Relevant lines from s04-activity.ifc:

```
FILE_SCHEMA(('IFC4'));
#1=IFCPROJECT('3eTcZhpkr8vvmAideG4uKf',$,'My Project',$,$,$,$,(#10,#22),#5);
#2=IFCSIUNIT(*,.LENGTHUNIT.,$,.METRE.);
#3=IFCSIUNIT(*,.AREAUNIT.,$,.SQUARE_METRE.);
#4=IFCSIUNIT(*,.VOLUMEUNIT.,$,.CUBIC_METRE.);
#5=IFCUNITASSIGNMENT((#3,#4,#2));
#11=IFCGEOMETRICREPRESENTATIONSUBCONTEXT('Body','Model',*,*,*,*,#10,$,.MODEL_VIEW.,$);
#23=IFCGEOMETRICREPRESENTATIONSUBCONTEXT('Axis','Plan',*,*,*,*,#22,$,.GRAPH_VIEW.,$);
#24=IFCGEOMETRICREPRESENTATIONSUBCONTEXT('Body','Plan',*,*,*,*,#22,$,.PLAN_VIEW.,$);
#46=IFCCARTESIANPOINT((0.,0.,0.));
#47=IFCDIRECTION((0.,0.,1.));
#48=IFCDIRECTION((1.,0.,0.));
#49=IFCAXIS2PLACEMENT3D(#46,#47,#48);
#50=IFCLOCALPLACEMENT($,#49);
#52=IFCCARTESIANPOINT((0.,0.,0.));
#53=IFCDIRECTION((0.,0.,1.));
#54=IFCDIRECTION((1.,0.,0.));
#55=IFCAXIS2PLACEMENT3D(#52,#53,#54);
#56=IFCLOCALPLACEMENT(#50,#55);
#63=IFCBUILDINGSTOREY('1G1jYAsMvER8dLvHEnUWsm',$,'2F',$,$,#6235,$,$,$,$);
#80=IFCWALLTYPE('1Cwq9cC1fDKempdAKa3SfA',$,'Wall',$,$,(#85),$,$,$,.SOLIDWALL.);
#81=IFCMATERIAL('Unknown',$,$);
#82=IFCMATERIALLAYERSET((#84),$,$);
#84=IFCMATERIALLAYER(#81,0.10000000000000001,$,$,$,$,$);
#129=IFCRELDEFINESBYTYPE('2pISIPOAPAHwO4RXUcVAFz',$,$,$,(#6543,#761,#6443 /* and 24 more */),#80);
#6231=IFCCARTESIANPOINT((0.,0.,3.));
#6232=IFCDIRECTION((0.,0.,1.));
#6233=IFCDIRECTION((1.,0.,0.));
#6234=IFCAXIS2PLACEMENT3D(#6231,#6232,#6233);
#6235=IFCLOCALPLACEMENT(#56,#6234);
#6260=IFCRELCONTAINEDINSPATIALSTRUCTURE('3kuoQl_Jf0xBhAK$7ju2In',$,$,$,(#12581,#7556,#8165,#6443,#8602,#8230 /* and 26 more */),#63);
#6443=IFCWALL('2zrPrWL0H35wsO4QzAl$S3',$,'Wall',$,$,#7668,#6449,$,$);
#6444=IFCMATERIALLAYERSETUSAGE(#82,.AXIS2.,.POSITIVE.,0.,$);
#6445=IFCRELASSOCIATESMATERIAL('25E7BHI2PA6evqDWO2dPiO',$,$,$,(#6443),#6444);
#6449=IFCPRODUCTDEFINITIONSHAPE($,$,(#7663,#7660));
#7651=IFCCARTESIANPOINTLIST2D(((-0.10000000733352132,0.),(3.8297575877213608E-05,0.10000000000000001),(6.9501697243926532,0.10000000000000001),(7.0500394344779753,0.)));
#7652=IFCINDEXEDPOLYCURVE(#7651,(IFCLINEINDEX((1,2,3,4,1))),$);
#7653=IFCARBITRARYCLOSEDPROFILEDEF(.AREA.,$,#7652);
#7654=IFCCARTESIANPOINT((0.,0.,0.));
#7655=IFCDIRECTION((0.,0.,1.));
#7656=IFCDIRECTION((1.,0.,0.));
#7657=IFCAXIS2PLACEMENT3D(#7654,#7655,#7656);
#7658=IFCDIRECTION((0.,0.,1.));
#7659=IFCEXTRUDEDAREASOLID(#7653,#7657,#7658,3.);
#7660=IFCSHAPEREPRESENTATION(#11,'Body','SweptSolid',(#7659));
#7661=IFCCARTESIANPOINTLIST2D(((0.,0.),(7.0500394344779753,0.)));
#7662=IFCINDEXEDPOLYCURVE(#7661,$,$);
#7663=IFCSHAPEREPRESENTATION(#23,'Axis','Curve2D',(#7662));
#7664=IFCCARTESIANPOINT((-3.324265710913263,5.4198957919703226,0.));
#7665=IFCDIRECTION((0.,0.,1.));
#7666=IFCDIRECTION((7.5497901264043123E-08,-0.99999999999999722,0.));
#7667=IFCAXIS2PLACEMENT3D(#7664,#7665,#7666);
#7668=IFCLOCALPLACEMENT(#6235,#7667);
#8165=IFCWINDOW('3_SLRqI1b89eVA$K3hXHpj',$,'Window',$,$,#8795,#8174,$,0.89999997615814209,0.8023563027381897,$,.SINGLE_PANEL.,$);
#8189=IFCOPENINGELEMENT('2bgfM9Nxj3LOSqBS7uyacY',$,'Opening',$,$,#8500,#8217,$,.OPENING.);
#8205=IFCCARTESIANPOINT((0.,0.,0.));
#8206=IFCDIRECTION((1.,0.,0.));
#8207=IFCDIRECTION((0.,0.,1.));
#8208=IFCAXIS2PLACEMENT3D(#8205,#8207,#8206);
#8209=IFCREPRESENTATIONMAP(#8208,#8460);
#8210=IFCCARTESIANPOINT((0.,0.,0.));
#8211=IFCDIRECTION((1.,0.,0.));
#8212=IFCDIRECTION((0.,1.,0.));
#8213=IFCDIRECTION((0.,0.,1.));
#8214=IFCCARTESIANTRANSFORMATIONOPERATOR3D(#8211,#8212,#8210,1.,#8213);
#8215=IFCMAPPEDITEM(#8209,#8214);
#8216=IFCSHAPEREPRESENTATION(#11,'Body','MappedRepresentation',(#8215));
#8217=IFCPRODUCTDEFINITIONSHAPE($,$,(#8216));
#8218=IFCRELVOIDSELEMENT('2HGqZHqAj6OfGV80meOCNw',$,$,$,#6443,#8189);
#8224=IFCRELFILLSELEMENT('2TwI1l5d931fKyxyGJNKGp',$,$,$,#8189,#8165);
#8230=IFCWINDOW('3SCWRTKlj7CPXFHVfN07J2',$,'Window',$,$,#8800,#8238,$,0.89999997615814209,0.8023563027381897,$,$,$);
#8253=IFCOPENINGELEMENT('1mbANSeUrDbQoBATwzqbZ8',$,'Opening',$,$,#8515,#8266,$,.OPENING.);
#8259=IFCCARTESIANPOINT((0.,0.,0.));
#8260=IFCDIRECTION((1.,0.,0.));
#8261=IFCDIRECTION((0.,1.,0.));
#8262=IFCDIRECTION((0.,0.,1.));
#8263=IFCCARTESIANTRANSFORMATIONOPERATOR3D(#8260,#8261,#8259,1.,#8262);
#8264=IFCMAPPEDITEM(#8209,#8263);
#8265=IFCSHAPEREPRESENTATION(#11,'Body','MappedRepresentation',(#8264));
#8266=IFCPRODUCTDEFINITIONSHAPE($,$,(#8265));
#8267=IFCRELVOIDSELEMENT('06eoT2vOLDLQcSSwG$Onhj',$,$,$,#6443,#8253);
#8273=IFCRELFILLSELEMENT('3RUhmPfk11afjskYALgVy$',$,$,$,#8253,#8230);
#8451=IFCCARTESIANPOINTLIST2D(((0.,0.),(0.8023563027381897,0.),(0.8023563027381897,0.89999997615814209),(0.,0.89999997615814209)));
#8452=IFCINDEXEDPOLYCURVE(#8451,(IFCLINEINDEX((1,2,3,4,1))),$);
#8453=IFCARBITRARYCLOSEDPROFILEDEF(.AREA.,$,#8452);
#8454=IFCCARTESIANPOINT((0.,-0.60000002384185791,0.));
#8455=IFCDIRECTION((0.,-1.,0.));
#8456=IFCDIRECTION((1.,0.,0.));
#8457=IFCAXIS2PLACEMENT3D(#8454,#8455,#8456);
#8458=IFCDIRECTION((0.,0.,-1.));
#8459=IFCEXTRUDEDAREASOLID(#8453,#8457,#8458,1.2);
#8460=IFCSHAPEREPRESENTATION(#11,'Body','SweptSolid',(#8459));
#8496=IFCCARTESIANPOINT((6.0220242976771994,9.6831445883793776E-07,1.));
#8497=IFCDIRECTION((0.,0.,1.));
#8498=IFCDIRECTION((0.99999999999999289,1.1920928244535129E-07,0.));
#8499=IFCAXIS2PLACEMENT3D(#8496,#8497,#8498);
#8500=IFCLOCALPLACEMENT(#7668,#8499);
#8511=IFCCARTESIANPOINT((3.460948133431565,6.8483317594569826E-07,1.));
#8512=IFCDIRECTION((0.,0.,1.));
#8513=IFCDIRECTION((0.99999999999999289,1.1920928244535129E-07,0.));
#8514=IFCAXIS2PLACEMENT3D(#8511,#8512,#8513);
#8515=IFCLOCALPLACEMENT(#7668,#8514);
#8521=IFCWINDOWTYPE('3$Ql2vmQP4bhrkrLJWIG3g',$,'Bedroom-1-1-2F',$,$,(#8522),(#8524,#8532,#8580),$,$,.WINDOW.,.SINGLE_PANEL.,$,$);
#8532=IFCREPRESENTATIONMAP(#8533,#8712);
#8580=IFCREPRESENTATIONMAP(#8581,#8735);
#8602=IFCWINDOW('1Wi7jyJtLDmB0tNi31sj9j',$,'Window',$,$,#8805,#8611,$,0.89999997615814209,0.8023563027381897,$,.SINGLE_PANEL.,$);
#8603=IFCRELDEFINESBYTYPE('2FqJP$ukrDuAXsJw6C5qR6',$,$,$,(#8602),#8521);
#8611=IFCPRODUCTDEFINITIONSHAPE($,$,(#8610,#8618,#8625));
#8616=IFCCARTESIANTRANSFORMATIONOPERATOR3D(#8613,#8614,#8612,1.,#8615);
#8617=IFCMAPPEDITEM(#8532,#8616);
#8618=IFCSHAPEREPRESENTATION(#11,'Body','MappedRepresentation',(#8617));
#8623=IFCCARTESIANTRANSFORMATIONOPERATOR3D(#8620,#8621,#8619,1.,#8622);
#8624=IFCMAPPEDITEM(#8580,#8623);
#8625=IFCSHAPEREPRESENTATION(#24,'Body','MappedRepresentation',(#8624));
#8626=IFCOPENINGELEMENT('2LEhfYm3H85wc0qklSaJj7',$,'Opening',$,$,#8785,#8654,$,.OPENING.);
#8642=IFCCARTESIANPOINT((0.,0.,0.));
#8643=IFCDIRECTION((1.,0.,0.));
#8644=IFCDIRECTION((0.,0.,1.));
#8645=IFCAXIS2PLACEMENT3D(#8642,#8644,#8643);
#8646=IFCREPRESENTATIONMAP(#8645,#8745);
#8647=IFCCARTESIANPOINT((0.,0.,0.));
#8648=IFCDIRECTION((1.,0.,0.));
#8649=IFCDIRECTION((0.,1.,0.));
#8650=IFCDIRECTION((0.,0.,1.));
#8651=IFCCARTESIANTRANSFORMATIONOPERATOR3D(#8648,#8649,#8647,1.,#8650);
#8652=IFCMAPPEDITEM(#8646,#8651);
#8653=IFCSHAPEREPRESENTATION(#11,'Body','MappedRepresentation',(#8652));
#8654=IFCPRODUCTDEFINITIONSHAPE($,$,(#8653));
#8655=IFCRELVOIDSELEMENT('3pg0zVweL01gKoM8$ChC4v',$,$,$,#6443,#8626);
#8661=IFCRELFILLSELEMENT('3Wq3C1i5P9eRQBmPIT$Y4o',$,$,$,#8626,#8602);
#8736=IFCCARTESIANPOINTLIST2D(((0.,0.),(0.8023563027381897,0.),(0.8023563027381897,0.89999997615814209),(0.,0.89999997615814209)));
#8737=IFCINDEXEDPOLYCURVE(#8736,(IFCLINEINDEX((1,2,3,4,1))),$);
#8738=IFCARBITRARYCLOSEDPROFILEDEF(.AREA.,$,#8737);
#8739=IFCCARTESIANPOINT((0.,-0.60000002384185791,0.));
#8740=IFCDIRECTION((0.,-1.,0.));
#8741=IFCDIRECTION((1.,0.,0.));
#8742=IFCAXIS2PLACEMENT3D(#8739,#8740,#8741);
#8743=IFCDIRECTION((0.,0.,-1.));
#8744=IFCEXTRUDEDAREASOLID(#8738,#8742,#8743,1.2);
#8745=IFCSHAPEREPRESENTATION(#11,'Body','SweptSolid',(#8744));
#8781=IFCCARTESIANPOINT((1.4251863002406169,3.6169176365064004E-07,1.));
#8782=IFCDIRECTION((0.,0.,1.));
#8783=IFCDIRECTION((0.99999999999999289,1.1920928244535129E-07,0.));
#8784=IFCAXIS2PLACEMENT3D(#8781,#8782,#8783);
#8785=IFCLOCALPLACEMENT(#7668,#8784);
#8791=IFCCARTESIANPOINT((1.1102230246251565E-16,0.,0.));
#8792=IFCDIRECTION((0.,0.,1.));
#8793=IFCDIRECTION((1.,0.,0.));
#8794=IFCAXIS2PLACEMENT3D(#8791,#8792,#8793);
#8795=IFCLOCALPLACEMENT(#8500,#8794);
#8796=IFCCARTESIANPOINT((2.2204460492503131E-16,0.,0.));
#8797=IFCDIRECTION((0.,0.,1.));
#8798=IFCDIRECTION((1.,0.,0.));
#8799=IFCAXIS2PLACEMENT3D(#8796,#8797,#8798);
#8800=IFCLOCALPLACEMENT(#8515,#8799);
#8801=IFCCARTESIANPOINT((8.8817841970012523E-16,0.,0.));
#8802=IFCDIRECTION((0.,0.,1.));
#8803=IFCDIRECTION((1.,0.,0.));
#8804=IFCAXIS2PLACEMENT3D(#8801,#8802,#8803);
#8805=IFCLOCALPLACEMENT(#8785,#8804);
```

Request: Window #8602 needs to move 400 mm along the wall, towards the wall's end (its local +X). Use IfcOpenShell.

```python
import ifcopenshell
import ifcopenshell.api.geometry
import ifcopenshell.util.placement
import ifcopenshell.util.unit

model = ifcopenshell.open("s04-activity.ifc")
unit_scale = ifcopenshell.util.unit.calculate_unit_scale(model)

window = model.by_guid("1Wi7jyJtLDmB0tNi31sj9j")
opening = window.FillsVoids[0].RelatingOpeningElement
wall = opening.VoidsElements[0].RelatingBuildingElement

wall_matrix = ifcopenshell.util.placement.get_local_placement(wall.ObjectPlacement)
shift = wall_matrix[:3, 0] * 0.4 / unit_scale
before = ifcopenshell.util.placement.get_local_placement(window.ObjectPlacement)[:3, 3].copy()

# The window is placed relative to its opening, so it follows when the opening moves.
matrix = ifcopenshell.util.placement.get_local_placement(opening.ObjectPlacement)
matrix[:3, 3] += shift
ifcopenshell.api.geometry.edit_object_placement(
    model, product=opening, matrix=matrix, is_si=False, should_transform_children=True
)

after = ifcopenshell.util.placement.get_local_placement(window.ObjectPlacement)[:3, 3]
print("window moved by", (after - before).round(3) + 0.0)

model.write("s04-activity_v2.ifc")
```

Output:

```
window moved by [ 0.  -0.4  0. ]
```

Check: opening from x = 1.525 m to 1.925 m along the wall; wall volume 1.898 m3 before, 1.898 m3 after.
